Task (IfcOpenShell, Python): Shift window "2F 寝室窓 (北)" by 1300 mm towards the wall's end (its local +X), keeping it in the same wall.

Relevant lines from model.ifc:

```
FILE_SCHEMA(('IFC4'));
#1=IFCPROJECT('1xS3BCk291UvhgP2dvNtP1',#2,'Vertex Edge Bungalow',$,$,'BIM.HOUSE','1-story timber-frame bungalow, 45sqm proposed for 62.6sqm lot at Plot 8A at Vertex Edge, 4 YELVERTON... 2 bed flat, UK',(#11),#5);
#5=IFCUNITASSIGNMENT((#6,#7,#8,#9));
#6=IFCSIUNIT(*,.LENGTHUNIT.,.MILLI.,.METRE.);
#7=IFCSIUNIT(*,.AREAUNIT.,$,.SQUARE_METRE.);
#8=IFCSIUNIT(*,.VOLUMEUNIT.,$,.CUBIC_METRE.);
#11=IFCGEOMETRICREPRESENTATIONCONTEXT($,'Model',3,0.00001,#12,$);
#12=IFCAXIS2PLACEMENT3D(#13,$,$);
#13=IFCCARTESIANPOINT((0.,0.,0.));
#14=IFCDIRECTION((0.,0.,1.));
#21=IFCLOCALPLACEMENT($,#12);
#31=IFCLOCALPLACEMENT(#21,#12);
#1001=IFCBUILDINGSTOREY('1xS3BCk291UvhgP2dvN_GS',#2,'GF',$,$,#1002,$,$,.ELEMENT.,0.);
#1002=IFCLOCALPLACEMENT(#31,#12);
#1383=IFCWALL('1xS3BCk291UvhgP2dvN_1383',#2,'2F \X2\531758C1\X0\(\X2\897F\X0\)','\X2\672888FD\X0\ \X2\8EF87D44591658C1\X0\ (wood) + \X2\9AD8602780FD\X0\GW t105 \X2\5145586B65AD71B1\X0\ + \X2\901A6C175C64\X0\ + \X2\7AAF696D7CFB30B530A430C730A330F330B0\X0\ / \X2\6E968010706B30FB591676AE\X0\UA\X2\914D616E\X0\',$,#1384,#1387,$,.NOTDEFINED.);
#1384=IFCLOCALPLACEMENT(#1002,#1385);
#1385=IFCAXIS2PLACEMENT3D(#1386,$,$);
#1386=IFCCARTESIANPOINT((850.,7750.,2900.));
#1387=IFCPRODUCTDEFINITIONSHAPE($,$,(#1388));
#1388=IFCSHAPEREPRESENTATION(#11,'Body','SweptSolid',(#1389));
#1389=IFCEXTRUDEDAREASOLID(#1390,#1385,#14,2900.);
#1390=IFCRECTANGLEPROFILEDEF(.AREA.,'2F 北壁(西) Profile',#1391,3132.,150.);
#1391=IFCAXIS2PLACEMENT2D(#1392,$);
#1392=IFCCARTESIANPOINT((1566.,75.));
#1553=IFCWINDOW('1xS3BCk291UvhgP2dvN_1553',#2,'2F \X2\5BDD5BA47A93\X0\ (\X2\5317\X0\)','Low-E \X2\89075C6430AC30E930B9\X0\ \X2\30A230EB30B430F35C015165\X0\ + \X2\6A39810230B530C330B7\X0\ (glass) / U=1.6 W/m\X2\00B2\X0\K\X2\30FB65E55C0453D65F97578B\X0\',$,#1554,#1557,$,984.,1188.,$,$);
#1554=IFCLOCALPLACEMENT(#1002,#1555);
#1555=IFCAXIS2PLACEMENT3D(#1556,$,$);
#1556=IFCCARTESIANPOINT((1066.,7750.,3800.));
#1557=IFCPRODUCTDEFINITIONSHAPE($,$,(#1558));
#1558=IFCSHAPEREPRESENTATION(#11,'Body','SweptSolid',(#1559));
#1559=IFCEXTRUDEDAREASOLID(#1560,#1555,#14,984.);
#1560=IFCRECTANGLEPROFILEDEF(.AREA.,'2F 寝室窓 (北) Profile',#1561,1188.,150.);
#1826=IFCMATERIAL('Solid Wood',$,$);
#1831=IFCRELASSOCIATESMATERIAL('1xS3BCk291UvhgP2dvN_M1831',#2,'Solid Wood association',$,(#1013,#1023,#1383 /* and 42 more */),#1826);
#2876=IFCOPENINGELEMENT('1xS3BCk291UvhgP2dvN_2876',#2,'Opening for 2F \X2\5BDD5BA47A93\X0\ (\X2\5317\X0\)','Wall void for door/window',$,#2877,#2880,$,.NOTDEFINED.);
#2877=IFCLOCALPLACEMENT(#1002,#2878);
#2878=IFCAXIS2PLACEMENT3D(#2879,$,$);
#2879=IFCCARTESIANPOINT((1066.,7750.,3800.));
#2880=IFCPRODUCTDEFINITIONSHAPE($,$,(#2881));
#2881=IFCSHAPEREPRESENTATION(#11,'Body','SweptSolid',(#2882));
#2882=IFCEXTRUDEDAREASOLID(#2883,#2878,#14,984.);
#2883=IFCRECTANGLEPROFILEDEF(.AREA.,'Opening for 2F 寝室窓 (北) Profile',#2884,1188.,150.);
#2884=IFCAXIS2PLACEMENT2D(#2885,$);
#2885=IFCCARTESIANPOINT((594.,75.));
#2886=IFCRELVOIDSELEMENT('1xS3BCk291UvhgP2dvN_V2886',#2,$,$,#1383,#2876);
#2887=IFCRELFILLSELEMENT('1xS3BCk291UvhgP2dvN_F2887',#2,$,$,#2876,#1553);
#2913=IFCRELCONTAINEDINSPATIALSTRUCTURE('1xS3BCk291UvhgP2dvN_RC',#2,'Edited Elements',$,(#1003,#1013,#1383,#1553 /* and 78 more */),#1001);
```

```python
import ifcopenshell
import ifcopenshell.api.geometry
import ifcopenshell.util.placement
import ifcopenshell.util.unit

model = ifcopenshell.open("model.ifc")
unit_scale = ifcopenshell.util.unit.calculate_unit_scale(model)

window = model.by_guid("1xS3BCk291UvhgP2dvN_1553")
opening = window.FillsVoids[0].RelatingOpeningElement
wall = opening.VoidsElements[0].RelatingBuildingElement

wall_matrix = ifcopenshell.util.placement.get_local_placement(wall.ObjectPlacement)
shift = wall_matrix[:3, 0] * 1.3 / unit_scale
before = ifcopenshell.util.placement.get_local_placement(window.ObjectPlacement)[:3, 3].copy()

# The window is not placed relative to its opening, so move both.
for product in (opening, window):
    matrix = ifcopenshell.util.placement.get_local_placement(product.ObjectPlacement)
    matrix[:3, 3] += shift
    ifcopenshell.api.geometry.edit_object_placement(model, product=product, matrix=matrix, is_si=False)

after = ifcopenshell.util.placement.get_local_placement(window.ObjectPlacement)[:3, 3]
print("window moved by", (after - before).round(3) + 0.0)

model.write("model_v2.ifc")
```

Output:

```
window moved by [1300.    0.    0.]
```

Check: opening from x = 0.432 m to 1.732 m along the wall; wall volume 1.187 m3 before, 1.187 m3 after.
